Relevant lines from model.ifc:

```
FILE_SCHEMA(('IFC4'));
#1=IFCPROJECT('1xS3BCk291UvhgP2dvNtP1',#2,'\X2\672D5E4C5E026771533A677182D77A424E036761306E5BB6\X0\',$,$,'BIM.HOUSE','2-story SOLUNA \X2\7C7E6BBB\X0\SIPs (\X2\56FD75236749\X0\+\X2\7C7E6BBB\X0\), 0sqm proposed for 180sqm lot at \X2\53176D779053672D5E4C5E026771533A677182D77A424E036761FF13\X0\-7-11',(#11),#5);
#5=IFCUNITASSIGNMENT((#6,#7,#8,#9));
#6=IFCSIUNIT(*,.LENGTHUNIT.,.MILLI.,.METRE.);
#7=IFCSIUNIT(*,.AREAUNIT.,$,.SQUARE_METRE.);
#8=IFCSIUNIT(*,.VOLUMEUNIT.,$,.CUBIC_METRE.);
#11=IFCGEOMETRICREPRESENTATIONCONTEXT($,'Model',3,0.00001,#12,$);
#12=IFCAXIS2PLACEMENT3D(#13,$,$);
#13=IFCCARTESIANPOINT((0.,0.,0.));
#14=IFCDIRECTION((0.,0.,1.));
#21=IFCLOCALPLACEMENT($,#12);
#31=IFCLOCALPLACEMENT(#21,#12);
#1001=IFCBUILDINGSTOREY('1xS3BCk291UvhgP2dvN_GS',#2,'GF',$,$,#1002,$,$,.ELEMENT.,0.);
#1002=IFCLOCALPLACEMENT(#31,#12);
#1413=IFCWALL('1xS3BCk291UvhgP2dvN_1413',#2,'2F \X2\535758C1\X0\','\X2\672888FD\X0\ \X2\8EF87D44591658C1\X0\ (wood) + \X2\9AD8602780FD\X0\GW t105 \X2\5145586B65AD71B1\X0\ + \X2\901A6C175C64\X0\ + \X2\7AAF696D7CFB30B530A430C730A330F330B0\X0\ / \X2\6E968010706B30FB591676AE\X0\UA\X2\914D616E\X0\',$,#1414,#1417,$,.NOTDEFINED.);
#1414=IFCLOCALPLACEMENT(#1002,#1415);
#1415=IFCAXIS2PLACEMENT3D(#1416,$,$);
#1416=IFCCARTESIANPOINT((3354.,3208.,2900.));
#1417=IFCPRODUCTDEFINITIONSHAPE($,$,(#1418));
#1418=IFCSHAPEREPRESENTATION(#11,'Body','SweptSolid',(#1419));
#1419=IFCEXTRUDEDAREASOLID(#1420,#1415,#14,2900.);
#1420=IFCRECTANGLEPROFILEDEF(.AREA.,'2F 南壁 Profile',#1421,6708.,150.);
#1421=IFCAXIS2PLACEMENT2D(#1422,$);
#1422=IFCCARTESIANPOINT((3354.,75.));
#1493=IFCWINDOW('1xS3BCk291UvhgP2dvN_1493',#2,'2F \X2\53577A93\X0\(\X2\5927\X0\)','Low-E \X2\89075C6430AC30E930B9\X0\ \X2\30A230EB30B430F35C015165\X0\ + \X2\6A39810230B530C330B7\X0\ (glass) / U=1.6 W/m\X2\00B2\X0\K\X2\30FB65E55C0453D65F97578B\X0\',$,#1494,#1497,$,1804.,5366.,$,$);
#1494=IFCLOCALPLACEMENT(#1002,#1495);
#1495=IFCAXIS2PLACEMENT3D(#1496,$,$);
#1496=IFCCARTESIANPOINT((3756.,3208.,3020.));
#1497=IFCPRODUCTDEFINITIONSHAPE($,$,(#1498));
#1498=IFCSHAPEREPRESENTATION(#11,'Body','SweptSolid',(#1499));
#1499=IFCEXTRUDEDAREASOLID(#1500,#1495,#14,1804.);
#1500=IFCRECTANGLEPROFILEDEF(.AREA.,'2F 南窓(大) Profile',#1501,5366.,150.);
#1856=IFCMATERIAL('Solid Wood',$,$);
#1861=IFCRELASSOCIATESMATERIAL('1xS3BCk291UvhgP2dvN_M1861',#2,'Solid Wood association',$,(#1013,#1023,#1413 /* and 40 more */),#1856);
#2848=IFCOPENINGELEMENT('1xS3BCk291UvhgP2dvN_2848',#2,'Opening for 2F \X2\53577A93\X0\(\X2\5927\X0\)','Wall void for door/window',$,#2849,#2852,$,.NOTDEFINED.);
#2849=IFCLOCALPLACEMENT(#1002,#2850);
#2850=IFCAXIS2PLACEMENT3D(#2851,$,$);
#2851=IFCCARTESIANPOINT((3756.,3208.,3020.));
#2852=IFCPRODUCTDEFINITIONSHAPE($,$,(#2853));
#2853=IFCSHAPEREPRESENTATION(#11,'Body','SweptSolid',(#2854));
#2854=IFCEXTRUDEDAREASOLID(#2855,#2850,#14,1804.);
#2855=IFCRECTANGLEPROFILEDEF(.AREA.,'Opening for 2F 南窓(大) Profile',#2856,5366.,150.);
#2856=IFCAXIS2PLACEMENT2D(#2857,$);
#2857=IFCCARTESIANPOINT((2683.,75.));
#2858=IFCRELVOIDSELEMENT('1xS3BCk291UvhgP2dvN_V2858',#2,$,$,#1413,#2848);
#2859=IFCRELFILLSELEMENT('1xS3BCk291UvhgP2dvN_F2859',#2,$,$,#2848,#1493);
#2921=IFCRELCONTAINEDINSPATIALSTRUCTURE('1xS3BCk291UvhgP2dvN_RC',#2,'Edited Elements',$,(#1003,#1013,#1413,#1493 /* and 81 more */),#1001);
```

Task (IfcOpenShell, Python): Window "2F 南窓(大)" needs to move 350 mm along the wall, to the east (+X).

```python
import ifcopenshell
import ifcopenshell.api.geometry
import ifcopenshell.util.placement

model = ifcopenshell.open("model.ifc")

window = model.by_guid("1xS3BCk291UvhgP2dvN_1493")
opening = window.FillsVoids[0].RelatingOpeningElement
wall = opening.VoidsElements[0].RelatingBuildingElement

wall_matrix = ifcopenshell.util.placement.get_local_placement(wall.ObjectPlacement)
shift = wall_matrix[:3, 0] * 350.0
before = ifcopenshell.util.placement.get_local_placement(window.ObjectPlacement)[:3, 3].copy()

# The window is not placed relative to its opening, so move both.
for product in (opening, window):
    matrix = ifcopenshell.util.placement.get_local_placement(product.ObjectPlacement)
    matrix[:3, 3] += shift
    ifcopenshell.api.geometry.edit_object_placement(model, product=product, matrix=matrix, is_si=False)

after = ifcopenshell.util.placement.get_local_placement(window.ObjectPlacement)[:3, 3]
print("window moved by", (after - before).round(3) + 0.0)

model.write("model_v2.ifc")
```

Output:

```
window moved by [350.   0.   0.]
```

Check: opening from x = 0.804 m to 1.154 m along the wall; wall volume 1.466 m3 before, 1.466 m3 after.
